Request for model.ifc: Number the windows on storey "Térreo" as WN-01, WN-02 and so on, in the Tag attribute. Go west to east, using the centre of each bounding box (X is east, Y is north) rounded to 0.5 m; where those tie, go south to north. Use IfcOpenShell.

First a look at what the model holds.

```python
import ifcopenshell
import ifcopenshell.util.element
import ifcopenshell.util.placement

model = ifcopenshell.open("model.ifc")
print(model.schema)
storey = next(s for s in model.by_type("IfcBuildingStorey") if s.Name == "Térreo")
windows = [e for e in ifcopenshell.util.element.get_decomposition(storey) if e.is_a("IfcWindow")]
for e in sorted(windows, key=lambda e: e.id()):
    origin = ifcopenshell.util.placement.get_local_placement(e.ObjectPlacement)[:3, 3]
    print(e.id(), e.Tag, e.Name, origin.round(2) + 0.0, sep=" | ")
```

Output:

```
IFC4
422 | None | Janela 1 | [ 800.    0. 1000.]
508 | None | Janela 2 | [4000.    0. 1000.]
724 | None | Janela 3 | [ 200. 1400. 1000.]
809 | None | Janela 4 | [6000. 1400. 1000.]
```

```python
import ifcopenshell
import ifcopenshell.geom
import ifcopenshell.util.element
import ifcopenshell.util.shape

model = ifcopenshell.open("model.ifc")
settings = ifcopenshell.geom.settings()
settings.set("use-world-coords", True)


def centre(element):
    shape = ifcopenshell.geom.create_shape(settings, element)
    return ifcopenshell.util.shape.get_bbox_centroid(shape.geometry)


storey = next(s for s in model.by_type("IfcBuildingStorey") if s.Name == "Térreo")
windows = [e for e in ifcopenshell.util.element.get_decomposition(storey) if e.is_a("IfcWindow")]

# Insertion points can sit at a corner or the storey origin, so sort by the geometry (in metres).
centres = {e: centre(e) for e in windows}
windows.sort(key=lambda e: (round(centres[e][0] / 0.5), centres[e][1]))

for i, e in enumerate(windows, start=1):
    number = f"WN-{i:02d}"
    e.Tag = number
    print(e.id(), number)

model.write("model_updated.ifc")
```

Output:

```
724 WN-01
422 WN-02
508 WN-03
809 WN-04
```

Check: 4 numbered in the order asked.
